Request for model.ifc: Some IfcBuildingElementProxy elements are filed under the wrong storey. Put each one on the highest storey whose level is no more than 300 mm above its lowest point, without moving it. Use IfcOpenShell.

First a look at what the model holds.

```python
import ifcopenshell
import ifcopenshell.util.element
import ifcopenshell.util.placement

model = ifcopenshell.open("model.ifc")
print(model.schema)
for storey in model.by_type("IfcBuildingStorey"):
    level = ifcopenshell.util.placement.get_storey_elevation(storey)
    count = sum(e.is_a("IfcBuildingElementProxy") for e in ifcopenshell.util.element.get_contained(storey))
    print(storey.id(), storey.Name, round(level, 3), count, sep=" | ")
```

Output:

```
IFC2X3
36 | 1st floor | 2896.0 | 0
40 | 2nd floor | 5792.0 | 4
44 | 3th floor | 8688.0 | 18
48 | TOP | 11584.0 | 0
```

```python
import ifcopenshell
import ifcopenshell.api.spatial
import ifcopenshell.geom
import ifcopenshell.util.element
import ifcopenshell.util.placement
import ifcopenshell.util.shape
import ifcopenshell.util.unit

model = ifcopenshell.open("model.ifc")
unit_scale = ifcopenshell.util.unit.calculate_unit_scale(model)
settings = ifcopenshell.geom.settings()

levels = sorted(
    ((ifcopenshell.util.placement.get_storey_elevation(s) * unit_scale, s) for s in model.by_type("IfcBuildingStorey")),
    key=lambda pair: pair[0],
)

for e in model.by_type("IfcBuildingElementProxy"):
    current = e.ContainedInStructure[0].RelatingStructure if e.ContainedInStructure else None
    if current is None or not current.is_a("IfcBuildingStorey"):
        continue
    shape = ifcopenshell.geom.create_shape(settings, e)
    bottom = ifcopenshell.util.shape.get_shape_bottom_elevation(shape, shape.geometry)
    below = [s for level, s in levels if level <= bottom + 0.3]
    storey = below[-1] if below else levels[0][1]
    if storey != current:
        # assign_container keeps the world position.
        ifcopenshell.api.spatial.assign_container(model, products=[e], relating_structure=storey)
        print(e.id(), current.Name, "->", storey.Name)

model.write("model_edited.ifc")
```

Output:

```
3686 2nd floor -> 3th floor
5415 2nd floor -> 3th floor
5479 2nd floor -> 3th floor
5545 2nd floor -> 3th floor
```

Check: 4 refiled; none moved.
